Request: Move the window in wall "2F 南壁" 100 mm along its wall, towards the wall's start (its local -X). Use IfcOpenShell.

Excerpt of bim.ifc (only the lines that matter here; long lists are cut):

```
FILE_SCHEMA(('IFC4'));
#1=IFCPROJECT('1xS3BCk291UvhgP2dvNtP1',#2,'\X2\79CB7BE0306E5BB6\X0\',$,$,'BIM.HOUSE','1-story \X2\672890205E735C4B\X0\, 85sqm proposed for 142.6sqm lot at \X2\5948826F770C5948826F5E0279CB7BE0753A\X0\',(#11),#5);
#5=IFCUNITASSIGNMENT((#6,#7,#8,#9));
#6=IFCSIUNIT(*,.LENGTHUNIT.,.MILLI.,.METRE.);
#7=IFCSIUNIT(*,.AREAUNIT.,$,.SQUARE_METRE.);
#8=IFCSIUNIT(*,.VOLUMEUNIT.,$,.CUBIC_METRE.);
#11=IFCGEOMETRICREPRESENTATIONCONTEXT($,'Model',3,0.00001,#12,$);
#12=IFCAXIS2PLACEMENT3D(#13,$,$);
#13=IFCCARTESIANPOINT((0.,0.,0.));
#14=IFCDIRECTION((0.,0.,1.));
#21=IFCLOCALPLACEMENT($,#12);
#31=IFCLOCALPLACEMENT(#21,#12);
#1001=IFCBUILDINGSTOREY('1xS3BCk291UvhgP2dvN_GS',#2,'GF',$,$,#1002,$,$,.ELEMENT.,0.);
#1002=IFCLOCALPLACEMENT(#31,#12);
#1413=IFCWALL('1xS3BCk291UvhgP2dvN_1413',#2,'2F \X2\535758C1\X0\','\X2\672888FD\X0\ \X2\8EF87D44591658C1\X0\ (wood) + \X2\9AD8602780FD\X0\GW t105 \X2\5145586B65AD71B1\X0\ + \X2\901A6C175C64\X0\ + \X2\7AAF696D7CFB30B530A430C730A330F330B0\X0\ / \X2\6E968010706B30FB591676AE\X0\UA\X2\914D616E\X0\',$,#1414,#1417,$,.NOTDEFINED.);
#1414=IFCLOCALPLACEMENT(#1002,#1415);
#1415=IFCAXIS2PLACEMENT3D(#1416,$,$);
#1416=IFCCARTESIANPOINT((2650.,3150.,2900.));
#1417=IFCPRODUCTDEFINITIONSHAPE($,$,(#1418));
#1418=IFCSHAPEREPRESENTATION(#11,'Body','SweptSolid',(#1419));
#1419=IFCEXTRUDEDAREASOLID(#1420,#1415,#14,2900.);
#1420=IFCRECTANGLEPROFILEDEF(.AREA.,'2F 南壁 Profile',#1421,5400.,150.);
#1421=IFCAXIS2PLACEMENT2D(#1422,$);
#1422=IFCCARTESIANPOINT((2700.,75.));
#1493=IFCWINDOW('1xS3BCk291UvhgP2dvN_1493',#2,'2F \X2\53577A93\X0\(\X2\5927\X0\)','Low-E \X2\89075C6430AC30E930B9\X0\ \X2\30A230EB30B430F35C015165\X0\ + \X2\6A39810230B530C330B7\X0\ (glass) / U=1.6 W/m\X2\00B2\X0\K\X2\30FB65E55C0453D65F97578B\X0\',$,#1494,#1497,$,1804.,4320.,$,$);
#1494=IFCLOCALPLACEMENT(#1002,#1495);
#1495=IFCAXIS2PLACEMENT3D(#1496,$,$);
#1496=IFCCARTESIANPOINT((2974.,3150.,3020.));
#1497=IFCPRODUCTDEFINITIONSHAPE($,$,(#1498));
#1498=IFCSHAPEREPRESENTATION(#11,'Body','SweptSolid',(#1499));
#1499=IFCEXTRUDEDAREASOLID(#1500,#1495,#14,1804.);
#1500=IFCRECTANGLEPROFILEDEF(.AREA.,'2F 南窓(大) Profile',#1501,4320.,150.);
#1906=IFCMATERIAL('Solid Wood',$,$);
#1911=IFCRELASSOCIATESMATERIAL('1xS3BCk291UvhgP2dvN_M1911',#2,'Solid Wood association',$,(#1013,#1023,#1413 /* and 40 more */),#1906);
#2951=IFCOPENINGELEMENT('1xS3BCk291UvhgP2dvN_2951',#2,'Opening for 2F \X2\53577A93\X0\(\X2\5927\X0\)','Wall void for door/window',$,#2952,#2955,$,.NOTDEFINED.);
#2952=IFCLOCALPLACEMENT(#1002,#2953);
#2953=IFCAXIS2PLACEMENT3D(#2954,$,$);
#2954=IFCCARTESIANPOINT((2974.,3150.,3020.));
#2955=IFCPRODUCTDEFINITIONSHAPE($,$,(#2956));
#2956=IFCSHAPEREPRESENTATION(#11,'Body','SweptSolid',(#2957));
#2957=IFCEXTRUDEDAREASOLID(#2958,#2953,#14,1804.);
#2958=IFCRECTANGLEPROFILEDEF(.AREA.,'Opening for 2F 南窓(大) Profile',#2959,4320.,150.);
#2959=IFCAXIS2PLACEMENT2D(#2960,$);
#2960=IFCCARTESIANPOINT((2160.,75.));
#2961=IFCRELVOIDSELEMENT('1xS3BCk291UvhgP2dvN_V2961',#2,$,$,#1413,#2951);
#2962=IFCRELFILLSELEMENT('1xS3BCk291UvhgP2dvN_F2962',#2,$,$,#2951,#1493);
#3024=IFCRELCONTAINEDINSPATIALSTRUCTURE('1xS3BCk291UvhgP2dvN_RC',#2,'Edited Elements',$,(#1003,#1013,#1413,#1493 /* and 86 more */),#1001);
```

```python
import ifcopenshell
import ifcopenshell.api.geometry
import ifcopenshell.util.placement
import ifcopenshell.util.unit

model = ifcopenshell.open("bim.ifc")
unit_scale = ifcopenshell.util.unit.calculate_unit_scale(model)

window = model.by_id(1493)
opening = window.FillsVoids[0].RelatingOpeningElement
wall = opening.VoidsElements[0].RelatingBuildingElement

wall_matrix = ifcopenshell.util.placement.get_local_placement(wall.ObjectPlacement)
shift = wall_matrix[:3, 0] * -0.1 / unit_scale
before = ifcopenshell.util.placement.get_local_placement(window.ObjectPlacement)[:3, 3].copy()

# The window is not placed relative to its opening, so move both.
for product in (opening, window):
    matrix = ifcopenshell.util.placement.get_local_placement(product.ObjectPlacement)
    matrix[:3, 3] += shift
    ifcopenshell.api.geometry.edit_object_placement(model, product=product, matrix=matrix, is_si=False)

after = ifcopenshell.util.placement.get_local_placement(window.ObjectPlacement)[:3, 3]
print("window moved by", (after - before).round(3) + 0.0)

model.write("bim_v2.ifc")
```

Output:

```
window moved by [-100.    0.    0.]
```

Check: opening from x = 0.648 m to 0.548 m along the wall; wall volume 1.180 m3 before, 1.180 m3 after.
